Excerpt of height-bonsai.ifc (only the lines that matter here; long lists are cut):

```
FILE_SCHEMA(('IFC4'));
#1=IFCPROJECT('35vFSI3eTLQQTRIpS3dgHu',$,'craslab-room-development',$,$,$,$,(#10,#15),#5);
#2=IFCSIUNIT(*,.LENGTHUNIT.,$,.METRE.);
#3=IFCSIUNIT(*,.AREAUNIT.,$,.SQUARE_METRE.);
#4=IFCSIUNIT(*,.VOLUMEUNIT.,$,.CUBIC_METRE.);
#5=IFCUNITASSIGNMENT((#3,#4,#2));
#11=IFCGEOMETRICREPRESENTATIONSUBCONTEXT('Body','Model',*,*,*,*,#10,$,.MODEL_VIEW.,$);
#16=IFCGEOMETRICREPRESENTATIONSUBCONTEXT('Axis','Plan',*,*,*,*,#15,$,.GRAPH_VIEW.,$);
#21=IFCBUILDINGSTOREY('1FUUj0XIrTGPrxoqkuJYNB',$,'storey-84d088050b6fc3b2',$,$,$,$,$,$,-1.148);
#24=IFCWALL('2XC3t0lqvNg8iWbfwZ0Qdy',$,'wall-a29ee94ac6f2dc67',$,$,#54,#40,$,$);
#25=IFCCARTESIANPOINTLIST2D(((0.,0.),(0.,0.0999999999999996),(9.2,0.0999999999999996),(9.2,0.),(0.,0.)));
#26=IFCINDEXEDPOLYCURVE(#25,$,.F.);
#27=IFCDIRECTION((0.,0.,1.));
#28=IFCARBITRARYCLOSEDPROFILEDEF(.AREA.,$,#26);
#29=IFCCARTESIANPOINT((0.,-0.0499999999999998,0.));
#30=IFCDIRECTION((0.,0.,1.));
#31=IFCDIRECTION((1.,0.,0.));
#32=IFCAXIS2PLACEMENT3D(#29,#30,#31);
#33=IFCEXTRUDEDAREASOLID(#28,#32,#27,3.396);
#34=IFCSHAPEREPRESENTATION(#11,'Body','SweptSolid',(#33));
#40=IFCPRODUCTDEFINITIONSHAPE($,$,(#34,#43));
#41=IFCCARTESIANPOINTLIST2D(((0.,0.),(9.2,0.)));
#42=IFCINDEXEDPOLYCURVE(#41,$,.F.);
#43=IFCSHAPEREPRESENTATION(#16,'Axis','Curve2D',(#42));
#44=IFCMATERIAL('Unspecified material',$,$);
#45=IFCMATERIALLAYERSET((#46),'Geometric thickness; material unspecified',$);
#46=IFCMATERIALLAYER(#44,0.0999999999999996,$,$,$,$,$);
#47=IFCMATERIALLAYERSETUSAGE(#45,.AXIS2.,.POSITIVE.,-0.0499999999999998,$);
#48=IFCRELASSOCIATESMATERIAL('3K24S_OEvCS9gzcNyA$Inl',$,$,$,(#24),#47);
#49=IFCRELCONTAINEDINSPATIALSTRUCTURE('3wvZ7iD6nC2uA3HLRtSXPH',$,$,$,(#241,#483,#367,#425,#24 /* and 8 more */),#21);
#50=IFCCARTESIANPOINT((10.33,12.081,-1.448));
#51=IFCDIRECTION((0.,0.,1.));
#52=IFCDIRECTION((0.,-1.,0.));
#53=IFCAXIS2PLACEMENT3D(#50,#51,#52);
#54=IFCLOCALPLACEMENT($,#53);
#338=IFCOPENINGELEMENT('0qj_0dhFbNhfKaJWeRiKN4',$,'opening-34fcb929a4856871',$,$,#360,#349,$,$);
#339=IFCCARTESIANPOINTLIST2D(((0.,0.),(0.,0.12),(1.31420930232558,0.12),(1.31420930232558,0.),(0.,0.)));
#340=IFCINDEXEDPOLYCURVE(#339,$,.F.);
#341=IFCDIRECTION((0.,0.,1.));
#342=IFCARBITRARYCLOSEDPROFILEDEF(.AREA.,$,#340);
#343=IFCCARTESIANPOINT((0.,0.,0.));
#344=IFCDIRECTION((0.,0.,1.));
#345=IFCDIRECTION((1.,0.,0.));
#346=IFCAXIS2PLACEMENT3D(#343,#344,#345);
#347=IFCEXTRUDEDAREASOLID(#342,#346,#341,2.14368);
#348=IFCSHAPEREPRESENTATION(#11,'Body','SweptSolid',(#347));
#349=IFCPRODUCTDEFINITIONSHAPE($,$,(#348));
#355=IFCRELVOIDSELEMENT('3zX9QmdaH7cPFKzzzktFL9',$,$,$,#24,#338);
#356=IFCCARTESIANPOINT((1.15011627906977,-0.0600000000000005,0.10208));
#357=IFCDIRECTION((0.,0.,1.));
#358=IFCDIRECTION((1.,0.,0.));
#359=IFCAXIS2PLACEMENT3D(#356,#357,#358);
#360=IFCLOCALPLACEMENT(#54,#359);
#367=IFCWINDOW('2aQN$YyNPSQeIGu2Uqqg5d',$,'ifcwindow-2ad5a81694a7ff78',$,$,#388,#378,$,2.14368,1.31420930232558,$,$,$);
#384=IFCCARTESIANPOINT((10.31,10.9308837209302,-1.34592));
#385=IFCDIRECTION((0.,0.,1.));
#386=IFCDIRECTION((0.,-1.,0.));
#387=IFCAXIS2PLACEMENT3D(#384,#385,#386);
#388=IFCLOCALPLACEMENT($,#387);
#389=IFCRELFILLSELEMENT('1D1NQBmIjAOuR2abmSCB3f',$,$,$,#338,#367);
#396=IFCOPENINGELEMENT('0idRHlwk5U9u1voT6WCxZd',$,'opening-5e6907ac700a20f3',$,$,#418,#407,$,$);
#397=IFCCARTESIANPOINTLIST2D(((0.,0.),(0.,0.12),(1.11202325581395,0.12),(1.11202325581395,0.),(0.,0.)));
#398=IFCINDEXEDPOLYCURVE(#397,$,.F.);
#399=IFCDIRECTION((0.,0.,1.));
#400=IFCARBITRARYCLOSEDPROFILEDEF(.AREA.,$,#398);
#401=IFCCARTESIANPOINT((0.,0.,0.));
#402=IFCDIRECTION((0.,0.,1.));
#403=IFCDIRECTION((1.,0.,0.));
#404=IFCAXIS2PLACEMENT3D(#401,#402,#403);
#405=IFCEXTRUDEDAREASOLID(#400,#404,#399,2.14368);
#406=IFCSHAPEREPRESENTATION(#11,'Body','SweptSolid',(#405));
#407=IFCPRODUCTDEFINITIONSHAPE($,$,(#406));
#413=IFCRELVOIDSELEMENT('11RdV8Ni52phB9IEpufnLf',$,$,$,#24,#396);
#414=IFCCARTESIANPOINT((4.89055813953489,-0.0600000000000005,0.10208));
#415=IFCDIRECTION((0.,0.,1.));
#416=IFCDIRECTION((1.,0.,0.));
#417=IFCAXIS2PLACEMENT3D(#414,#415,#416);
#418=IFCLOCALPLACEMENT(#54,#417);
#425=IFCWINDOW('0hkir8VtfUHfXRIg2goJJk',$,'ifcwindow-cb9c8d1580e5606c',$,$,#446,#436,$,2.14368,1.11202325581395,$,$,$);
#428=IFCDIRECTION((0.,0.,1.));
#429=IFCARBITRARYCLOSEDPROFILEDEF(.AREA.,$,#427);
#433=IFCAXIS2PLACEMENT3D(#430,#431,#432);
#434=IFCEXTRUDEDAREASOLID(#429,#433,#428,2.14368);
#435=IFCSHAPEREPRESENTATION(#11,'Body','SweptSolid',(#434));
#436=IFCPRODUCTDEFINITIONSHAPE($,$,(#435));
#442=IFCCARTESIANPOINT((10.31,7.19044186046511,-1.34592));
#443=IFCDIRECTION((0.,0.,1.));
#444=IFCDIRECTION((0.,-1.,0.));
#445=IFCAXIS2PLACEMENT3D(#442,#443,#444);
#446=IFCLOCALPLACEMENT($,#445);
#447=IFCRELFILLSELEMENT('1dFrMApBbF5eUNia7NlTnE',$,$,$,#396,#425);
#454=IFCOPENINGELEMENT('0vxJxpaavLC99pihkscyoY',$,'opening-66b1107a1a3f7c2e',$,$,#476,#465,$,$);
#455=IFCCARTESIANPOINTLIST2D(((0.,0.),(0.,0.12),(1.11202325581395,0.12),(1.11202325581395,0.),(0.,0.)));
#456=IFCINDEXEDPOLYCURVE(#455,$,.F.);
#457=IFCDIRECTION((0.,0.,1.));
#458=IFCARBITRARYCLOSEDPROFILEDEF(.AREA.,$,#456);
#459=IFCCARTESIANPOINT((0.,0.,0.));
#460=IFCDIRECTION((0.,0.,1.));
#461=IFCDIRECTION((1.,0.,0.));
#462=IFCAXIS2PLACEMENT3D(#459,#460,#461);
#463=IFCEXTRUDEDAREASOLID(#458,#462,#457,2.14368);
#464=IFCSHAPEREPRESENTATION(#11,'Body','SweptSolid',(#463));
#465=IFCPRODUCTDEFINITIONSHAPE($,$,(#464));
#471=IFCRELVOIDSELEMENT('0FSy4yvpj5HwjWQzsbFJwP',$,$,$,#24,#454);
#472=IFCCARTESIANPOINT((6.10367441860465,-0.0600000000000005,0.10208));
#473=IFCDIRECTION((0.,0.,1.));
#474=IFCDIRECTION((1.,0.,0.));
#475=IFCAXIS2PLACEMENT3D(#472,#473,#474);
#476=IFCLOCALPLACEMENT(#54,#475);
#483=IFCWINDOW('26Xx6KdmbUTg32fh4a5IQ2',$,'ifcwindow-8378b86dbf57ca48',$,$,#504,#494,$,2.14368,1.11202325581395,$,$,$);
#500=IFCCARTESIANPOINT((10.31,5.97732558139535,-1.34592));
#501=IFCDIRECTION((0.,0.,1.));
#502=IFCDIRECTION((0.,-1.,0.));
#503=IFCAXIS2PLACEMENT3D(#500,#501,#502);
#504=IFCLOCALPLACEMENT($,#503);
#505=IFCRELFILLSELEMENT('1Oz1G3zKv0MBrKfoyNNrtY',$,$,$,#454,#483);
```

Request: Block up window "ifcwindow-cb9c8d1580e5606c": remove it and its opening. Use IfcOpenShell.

```python
import ifcopenshell
import ifcopenshell.api.feature
import ifcopenshell.api.root
import ifcopenshell.geom
import ifcopenshell.util.shape

model = ifcopenshell.open("height-bonsai.ifc")
settings = ifcopenshell.geom.settings()


def volume(element):
    """Net volume in cubic metres, openings subtracted."""
    shape = ifcopenshell.geom.create_shape(settings, element)
    return ifcopenshell.util.shape.get_volume(shape.geometry)


window = model.by_guid("0hkir8VtfUHfXRIg2goJJk")
opening = window.FillsVoids[0].RelatingOpeningElement
wall = opening.VoidsElements[0].RelatingBuildingElement
before = volume(wall)

ifcopenshell.api.root.remove_product(model, product=window)
ifcopenshell.api.feature.remove_feature(model, feature=opening)

after = volume(wall)

print(f"wall volume {before:.3f} -> {after:.3f} m3")

model.write("height-bonsai_updated.ifc")
```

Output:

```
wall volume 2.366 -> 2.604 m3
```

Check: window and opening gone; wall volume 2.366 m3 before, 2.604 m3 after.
